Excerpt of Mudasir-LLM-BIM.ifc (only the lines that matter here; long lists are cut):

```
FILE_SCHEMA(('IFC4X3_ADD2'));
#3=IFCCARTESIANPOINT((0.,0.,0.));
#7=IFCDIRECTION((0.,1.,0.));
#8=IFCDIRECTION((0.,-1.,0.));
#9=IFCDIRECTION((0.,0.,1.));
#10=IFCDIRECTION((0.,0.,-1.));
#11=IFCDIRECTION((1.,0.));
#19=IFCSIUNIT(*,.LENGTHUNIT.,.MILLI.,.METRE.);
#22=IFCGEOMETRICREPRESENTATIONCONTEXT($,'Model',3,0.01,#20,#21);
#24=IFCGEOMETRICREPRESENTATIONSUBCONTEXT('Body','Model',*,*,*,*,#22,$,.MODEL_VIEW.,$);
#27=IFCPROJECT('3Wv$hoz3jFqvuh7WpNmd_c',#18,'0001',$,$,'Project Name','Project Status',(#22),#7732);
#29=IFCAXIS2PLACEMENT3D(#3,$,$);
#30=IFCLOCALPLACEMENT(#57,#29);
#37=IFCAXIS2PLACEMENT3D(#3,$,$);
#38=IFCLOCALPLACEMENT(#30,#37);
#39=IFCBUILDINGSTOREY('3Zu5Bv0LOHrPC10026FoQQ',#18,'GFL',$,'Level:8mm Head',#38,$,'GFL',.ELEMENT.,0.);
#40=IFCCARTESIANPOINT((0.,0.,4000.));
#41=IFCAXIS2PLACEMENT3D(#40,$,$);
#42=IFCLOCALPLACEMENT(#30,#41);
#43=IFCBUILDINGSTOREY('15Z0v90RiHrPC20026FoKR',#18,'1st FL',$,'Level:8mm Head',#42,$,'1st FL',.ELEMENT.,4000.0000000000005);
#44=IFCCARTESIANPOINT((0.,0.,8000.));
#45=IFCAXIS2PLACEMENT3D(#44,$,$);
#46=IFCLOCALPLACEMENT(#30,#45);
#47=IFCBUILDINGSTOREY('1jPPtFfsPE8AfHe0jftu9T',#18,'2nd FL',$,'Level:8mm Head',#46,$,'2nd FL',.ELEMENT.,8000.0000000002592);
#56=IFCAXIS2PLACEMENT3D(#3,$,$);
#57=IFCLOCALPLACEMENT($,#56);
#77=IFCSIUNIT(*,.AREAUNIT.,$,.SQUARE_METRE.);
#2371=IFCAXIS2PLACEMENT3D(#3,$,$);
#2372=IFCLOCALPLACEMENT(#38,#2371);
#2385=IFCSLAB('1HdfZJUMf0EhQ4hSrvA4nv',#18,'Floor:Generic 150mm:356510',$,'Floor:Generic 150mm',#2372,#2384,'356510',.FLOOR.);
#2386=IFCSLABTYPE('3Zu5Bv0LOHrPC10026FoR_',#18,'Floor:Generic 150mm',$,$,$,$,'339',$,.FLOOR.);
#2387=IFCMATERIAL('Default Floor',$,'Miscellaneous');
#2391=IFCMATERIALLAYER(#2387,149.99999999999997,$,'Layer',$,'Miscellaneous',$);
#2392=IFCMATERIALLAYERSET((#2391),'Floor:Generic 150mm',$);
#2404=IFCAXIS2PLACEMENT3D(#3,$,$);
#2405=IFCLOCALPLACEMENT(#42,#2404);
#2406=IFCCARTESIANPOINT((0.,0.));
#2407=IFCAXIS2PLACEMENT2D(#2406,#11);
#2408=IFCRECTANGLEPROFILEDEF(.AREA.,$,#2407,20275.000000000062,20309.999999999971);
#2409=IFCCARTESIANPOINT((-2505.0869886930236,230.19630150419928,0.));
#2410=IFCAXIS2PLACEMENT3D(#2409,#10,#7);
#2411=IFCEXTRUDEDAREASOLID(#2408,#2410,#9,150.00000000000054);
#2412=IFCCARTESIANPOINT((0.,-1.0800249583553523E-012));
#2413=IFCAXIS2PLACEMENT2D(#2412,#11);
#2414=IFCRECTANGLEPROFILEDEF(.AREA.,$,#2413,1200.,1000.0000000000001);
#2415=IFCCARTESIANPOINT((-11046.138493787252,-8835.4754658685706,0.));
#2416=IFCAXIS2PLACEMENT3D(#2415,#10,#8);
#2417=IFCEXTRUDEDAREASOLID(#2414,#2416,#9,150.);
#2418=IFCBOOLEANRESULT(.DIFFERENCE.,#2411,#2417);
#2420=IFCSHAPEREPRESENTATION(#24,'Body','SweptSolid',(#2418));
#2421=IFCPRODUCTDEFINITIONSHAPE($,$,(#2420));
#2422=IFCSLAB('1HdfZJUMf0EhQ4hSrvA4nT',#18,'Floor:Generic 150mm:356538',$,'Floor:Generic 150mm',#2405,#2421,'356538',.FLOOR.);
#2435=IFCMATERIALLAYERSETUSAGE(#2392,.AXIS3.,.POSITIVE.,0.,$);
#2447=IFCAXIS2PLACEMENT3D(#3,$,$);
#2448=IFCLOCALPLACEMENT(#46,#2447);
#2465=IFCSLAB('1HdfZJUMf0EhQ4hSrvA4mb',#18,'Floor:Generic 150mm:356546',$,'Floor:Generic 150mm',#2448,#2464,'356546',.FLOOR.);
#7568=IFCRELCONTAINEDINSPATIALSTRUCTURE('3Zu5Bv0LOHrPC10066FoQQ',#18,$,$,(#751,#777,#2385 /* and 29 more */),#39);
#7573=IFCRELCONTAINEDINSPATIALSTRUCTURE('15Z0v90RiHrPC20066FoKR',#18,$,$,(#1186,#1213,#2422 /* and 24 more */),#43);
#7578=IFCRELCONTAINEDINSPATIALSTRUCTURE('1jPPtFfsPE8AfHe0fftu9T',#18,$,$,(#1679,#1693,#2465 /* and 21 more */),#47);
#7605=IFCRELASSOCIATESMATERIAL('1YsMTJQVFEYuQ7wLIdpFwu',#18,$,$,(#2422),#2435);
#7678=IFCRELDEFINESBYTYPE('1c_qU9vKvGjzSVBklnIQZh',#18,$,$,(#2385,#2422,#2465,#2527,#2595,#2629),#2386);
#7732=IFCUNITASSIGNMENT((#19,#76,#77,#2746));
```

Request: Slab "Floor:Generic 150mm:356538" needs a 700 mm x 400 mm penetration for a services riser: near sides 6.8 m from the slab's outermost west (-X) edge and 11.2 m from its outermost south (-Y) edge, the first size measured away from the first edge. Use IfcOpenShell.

```python
import numpy as np
import ifcopenshell
import ifcopenshell.api.feature
import ifcopenshell.api.geometry
import ifcopenshell.api.root
import ifcopenshell.geom
import ifcopenshell.util.placement
import ifcopenshell.util.representation
import ifcopenshell.util.shape
import ifcopenshell.util.unit

model = ifcopenshell.open("Mudasir-LLM-BIM.ifc")
unit_scale = ifcopenshell.util.unit.calculate_unit_scale(model)
settings = ifcopenshell.geom.settings()


def volume(element):
    """Net volume in cubic metres, openings subtracted."""
    shape = ifcopenshell.geom.create_shape(settings, element)
    return ifcopenshell.util.shape.get_volume(shape.geometry)


slab = model.by_id(2422)
before = volume(slab)

# Extent in the slab's own axes, in metres. The edges named are its -X and -Y sides.
slab_shape = ifcopenshell.geom.create_shape(settings, slab)
vertices = ifcopenshell.util.shape.get_vertices(slab_shape.geometry)
x_min, y_min, bottom = vertices.min(axis=0)
top = vertices[:, 2].max()

opening = ifcopenshell.api.root.create_entity(model, ifc_class="IfcOpeningElement", name="Services riser opening", predefined_type="OPENING")
context = ifcopenshell.util.representation.get_context(model, "Model", "Body", "MODEL_VIEW")
width, depth = 0.7, 0.4
outline = [(0.0, 0.0), (width, 0.0), (width, depth), (0.0, depth), (0.0, 0.0)]
# Overshoot both faces by 50 mm so the cut is clean.
shape = ifcopenshell.api.geometry.add_slab_representation(
    model, context=context, depth=top - bottom + 0.1, polyline=outline
)
ifcopenshell.api.geometry.assign_representation(model, product=opening, representation=shape)

matrix = ifcopenshell.util.placement.get_local_placement(slab.ObjectPlacement)
matrix[:, 3] = matrix @ np.append(np.array([x_min + 6.8, y_min + 11.2, bottom - 0.05]) / unit_scale, 1.0)
ifcopenshell.api.geometry.edit_object_placement(model, product=opening, matrix=matrix, is_si=False)
ifcopenshell.api.feature.add_feature(model, feature=opening, element=slab)

after = volume(slab)

print(f"slab volume {before:.3f} -> {after:.3f} m3")

model.write("Mudasir-LLM-BIM_updated.ifc")
```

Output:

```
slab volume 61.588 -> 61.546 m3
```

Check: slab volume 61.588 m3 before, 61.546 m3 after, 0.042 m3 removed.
